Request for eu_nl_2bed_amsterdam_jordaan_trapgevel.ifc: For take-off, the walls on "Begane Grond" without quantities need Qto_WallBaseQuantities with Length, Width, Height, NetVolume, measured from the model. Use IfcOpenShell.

First a look at what the model holds.

```python
import ifcopenshell
import ifcopenshell.util.element
import ifcopenshell.util.unit

model = ifcopenshell.open("eu_nl_2bed_amsterdam_jordaan_trapgevel.ifc")
print(model.schema)
for unit_type in ("LENGTHUNIT", "AREAUNIT", "VOLUMEUNIT"):
    print(unit_type, ifcopenshell.util.unit.calculate_unit_scale(model, unit_type))
storey = next(s for s in model.by_type("IfcBuildingStorey") if s.Name == "Begane Grond")
walls = [e for e in ifcopenshell.util.element.get_decomposition(storey) if e.is_a("IfcWall")]
for e in sorted(walls, key=lambda e: e.id()):
    print(e.id(), e.is_a(), e.Name, list(ifcopenshell.util.element.get_psets(e, qtos_only=True)), sep=" | ")
```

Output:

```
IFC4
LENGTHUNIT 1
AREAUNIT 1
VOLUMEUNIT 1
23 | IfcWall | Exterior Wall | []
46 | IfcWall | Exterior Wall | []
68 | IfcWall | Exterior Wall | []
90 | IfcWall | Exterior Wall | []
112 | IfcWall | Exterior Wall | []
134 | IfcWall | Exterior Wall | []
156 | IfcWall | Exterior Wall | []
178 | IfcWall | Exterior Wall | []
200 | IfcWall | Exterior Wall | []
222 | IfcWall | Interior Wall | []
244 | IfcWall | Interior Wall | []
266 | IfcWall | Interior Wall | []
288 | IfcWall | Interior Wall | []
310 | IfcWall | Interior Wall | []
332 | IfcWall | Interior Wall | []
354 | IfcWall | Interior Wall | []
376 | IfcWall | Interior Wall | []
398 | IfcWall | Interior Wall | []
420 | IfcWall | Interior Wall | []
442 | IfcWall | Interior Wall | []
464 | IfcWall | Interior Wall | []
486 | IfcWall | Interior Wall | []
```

```python
import ifcopenshell
import ifcopenshell.api.pset
import ifcopenshell.geom
import ifcopenshell.util.element
import ifcopenshell.util.shape
import ifcopenshell.util.unit

model = ifcopenshell.open("eu_nl_2bed_amsterdam_jordaan_trapgevel.ifc")
unit_scale = ifcopenshell.util.unit.calculate_unit_scale(model)
volume_scale = ifcopenshell.util.unit.calculate_unit_scale(model, "VOLUMEUNIT")
settings = ifcopenshell.geom.settings()

storey = next(s for s in model.by_type("IfcBuildingStorey") if s.Name == "Begane Grond")
walls = [e for e in ifcopenshell.util.element.get_decomposition(storey) if e.is_a("IfcWall")]

for e in sorted(walls, key=lambda e: e.id()):
    if ifcopenshell.util.element.get_psets(e, qtos_only=True, should_inherit=False):
        continue
    # Geometry comes back in metres, in the element's own axes.
    shape = ifcopenshell.geom.create_shape(settings, e)
    values = {
        "Length": ifcopenshell.util.shape.get_x(shape.geometry) / unit_scale,
        "Width": ifcopenshell.util.shape.get_y(shape.geometry) / unit_scale,
        "Height": ifcopenshell.util.shape.get_z(shape.geometry) / unit_scale,
        "NetVolume": ifcopenshell.util.shape.get_volume(shape.geometry) / volume_scale,
    }
    qto = ifcopenshell.api.pset.add_qto(model, product=e, name="Qto_WallBaseQuantities")
    ifcopenshell.api.pset.edit_qto(model, qto=qto, properties=values)
    print(e.id(), {k: round(v, 3) for k, v in values.items()})

model.write("eu_nl_2bed_amsterdam_jordaan_trapgevel_updated.ifc")
```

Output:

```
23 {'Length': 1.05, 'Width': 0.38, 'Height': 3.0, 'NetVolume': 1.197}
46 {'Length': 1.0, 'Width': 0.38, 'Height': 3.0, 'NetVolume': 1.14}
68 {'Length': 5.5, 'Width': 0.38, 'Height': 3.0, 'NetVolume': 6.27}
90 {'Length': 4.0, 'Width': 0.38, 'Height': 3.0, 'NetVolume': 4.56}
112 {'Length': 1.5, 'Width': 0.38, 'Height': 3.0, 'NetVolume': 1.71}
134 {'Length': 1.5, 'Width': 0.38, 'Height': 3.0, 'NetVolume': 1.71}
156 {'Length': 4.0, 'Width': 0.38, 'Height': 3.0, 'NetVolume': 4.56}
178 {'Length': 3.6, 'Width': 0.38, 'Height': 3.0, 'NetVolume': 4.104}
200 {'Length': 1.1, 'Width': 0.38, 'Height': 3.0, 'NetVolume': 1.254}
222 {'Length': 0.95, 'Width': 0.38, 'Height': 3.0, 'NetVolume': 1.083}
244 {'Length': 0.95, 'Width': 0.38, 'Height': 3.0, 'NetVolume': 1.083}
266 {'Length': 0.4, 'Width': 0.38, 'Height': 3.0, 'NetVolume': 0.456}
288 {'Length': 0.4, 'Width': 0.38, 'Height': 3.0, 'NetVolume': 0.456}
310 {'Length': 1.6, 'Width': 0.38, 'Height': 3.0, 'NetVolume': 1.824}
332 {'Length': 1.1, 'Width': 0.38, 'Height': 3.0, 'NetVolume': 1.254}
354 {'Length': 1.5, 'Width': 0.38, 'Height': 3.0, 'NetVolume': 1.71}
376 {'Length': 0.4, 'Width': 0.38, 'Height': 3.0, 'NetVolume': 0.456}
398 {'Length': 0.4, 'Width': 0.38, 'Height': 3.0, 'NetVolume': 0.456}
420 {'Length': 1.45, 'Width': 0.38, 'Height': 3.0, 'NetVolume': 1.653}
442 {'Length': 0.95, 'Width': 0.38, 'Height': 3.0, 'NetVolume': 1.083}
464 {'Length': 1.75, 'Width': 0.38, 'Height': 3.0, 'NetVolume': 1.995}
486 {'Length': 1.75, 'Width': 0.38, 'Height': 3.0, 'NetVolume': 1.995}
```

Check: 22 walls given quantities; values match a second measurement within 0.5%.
